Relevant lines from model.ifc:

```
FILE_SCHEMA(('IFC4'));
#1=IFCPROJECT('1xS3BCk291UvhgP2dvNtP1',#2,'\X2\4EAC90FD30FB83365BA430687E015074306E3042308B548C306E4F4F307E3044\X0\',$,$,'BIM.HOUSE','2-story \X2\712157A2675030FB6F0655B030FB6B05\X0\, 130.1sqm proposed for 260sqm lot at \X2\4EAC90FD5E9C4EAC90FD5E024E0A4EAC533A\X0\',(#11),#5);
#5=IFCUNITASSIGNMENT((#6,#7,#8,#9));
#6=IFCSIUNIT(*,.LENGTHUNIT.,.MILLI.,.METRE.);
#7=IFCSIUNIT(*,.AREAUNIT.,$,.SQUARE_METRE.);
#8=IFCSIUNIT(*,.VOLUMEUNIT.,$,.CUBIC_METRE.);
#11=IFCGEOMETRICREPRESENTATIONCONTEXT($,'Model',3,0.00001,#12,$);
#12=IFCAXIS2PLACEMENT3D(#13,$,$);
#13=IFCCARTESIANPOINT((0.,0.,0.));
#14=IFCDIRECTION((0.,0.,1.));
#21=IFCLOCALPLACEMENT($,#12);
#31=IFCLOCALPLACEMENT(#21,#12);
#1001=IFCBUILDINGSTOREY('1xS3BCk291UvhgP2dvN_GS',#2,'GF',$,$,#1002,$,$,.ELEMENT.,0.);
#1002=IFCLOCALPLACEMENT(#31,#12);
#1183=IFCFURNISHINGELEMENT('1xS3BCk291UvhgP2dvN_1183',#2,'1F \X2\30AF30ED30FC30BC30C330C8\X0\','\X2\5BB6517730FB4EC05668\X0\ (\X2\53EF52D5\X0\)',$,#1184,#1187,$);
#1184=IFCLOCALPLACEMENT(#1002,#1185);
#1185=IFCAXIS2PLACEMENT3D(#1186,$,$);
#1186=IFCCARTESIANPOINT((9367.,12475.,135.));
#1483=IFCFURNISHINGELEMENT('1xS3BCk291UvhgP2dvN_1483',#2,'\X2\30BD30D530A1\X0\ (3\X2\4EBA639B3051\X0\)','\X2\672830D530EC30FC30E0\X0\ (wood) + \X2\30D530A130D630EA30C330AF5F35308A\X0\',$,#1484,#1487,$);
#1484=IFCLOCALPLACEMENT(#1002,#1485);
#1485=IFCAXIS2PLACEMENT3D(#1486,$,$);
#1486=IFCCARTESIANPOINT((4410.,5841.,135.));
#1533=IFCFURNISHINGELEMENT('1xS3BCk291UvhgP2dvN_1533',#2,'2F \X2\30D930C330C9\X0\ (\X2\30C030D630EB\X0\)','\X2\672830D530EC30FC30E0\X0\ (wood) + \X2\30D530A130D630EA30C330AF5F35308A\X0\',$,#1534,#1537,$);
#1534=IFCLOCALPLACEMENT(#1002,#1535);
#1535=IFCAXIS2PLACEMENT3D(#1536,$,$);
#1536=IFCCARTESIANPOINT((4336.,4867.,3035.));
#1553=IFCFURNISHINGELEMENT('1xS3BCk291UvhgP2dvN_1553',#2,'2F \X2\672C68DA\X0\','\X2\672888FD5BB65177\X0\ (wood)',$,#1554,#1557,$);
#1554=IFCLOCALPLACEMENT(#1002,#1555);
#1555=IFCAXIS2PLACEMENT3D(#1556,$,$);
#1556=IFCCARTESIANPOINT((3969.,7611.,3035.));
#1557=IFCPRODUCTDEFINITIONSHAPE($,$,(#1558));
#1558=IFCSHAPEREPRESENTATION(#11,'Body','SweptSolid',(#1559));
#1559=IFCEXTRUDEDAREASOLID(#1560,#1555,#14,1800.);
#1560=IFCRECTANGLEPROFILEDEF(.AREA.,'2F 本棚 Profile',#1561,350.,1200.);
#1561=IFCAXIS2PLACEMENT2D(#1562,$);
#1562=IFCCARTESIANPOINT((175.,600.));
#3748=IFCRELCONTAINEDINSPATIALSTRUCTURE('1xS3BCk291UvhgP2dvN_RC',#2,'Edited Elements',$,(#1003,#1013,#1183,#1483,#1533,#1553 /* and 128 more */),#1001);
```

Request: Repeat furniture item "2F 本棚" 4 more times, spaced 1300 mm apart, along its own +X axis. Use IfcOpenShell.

```python
import ifcopenshell
import ifcopenshell.api.geometry
import ifcopenshell.api.root
import ifcopenshell.util.element
import ifcopenshell.util.placement

model = ifcopenshell.open("model.ifc")


def reuse_history(source, copy):
    """copy_class also copies each property set's owner history, people and application; keep the originals."""
    for rel in copy.IsDefinedBy:
        if rel.is_a("IfcRelDefinesByProperties") and (history := rel.RelatingPropertyDefinition.OwnerHistory):
            rel.RelatingPropertyDefinition.OwnerHistory = source.OwnerHistory
            ifcopenshell.util.element.remove_deep2(model, history)


source = model.by_guid("1xS3BCk291UvhgP2dvN_1553")
base = ifcopenshell.util.placement.get_local_placement(source.ObjectPlacement)
step = base[:3, 0] * 1300.0

for i in range(1, 5):
    copy = ifcopenshell.api.root.copy_class(model, product=source)
    copy.Representation = ifcopenshell.util.element.copy_deep(
        model, source.Representation, exclude=["IfcGeometricRepresentationContext", "IfcRepresentationMap"]
    )
    reuse_history(source, copy)
    matrix = base.copy()
    matrix[:3, 3] += i * step
    print("added at", matrix[:3, 3].round(3) + 0.0)
    ifcopenshell.api.geometry.edit_object_placement(model, product=copy, matrix=matrix, is_si=False)

model.write("model_updated.ifc")
```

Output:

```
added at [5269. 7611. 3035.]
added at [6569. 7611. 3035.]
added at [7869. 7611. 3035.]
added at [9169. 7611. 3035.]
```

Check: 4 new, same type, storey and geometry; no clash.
